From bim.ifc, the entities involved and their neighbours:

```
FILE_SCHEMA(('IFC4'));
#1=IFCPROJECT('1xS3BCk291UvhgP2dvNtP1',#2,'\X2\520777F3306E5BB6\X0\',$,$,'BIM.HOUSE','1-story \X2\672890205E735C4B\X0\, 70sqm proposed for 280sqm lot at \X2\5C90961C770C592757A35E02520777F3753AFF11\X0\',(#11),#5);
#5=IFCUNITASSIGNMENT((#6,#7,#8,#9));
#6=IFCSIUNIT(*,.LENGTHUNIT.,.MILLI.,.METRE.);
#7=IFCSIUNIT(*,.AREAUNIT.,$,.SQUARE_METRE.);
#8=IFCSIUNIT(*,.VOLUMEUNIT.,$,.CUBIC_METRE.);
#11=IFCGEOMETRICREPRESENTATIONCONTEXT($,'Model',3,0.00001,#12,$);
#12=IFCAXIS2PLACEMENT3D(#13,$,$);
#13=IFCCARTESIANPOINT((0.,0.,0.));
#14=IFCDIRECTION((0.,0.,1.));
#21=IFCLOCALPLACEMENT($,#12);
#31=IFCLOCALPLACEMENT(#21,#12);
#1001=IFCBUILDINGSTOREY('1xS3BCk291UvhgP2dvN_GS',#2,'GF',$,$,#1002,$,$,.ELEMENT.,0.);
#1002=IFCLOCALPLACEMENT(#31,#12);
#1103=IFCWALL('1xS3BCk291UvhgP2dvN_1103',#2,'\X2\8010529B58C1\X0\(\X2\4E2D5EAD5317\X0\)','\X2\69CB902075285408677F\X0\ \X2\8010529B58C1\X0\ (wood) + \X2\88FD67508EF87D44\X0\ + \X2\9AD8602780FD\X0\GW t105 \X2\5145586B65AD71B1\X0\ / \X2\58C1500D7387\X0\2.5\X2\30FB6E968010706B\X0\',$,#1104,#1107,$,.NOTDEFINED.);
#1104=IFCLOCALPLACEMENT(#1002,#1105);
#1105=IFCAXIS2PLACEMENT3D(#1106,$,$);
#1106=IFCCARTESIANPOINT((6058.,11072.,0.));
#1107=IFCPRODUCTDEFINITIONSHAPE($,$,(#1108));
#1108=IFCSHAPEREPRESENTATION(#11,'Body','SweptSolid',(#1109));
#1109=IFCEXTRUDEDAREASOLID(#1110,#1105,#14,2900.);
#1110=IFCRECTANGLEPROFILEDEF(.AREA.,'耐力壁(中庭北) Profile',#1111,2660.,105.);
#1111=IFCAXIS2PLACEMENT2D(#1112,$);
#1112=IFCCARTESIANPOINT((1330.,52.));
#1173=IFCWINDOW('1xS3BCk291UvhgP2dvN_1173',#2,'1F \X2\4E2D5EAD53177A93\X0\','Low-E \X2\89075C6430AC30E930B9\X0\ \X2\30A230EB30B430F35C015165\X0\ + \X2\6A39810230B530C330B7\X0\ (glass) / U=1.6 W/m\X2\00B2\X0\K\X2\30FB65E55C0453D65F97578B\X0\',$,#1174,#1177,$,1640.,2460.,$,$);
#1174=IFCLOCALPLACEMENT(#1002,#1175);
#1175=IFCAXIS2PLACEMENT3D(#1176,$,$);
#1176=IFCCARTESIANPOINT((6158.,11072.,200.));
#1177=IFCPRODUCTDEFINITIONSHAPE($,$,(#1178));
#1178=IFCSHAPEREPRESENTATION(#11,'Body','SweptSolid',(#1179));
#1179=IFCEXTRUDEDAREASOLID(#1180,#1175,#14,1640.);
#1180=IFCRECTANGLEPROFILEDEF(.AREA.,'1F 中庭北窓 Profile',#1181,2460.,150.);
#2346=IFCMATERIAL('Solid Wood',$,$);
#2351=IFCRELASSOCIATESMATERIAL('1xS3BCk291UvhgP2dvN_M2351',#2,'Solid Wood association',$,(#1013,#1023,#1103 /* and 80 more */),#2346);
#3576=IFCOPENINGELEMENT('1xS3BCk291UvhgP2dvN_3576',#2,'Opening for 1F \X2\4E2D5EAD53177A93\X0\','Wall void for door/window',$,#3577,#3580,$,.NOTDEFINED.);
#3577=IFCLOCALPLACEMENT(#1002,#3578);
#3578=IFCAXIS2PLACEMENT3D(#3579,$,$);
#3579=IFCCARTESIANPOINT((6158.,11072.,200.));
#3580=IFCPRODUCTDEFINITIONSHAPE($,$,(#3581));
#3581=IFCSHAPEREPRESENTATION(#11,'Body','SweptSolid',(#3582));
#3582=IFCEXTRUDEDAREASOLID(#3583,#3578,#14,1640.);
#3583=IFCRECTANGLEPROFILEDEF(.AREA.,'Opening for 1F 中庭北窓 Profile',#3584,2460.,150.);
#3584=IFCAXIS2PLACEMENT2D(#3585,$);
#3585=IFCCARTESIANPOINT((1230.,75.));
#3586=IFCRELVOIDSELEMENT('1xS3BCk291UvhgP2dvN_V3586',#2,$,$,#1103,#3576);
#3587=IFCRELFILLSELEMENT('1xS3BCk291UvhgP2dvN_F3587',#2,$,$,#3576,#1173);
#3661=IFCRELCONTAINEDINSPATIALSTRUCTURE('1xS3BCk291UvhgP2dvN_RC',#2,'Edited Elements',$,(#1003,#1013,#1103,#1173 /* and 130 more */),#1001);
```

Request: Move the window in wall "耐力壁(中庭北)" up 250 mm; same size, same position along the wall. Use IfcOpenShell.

```python
import numpy as np
import ifcopenshell
import ifcopenshell.api.geometry
import ifcopenshell.util.placement
import ifcopenshell.util.unit

model = ifcopenshell.open("bim.ifc")
unit_scale = ifcopenshell.util.unit.calculate_unit_scale(model)

window = model.by_guid("1xS3BCk291UvhgP2dvN_1173")
opening = window.FillsVoids[0].RelatingOpeningElement
dz = 0.25 / unit_scale

shift = np.array([0.0, 0.0, dz])
# The window is not placed relative to its opening, so move both.
for product in (opening, window):
    matrix = ifcopenshell.util.placement.get_local_placement(product.ObjectPlacement)
    matrix[:3, 3] += shift
    ifcopenshell.api.geometry.edit_object_placement(model, product=product, matrix=matrix, is_si=False)

print(f"moved by {dz * unit_scale:+.3f} m")

model.write("bim-out.ifc")
```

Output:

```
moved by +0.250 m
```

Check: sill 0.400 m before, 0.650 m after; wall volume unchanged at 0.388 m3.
